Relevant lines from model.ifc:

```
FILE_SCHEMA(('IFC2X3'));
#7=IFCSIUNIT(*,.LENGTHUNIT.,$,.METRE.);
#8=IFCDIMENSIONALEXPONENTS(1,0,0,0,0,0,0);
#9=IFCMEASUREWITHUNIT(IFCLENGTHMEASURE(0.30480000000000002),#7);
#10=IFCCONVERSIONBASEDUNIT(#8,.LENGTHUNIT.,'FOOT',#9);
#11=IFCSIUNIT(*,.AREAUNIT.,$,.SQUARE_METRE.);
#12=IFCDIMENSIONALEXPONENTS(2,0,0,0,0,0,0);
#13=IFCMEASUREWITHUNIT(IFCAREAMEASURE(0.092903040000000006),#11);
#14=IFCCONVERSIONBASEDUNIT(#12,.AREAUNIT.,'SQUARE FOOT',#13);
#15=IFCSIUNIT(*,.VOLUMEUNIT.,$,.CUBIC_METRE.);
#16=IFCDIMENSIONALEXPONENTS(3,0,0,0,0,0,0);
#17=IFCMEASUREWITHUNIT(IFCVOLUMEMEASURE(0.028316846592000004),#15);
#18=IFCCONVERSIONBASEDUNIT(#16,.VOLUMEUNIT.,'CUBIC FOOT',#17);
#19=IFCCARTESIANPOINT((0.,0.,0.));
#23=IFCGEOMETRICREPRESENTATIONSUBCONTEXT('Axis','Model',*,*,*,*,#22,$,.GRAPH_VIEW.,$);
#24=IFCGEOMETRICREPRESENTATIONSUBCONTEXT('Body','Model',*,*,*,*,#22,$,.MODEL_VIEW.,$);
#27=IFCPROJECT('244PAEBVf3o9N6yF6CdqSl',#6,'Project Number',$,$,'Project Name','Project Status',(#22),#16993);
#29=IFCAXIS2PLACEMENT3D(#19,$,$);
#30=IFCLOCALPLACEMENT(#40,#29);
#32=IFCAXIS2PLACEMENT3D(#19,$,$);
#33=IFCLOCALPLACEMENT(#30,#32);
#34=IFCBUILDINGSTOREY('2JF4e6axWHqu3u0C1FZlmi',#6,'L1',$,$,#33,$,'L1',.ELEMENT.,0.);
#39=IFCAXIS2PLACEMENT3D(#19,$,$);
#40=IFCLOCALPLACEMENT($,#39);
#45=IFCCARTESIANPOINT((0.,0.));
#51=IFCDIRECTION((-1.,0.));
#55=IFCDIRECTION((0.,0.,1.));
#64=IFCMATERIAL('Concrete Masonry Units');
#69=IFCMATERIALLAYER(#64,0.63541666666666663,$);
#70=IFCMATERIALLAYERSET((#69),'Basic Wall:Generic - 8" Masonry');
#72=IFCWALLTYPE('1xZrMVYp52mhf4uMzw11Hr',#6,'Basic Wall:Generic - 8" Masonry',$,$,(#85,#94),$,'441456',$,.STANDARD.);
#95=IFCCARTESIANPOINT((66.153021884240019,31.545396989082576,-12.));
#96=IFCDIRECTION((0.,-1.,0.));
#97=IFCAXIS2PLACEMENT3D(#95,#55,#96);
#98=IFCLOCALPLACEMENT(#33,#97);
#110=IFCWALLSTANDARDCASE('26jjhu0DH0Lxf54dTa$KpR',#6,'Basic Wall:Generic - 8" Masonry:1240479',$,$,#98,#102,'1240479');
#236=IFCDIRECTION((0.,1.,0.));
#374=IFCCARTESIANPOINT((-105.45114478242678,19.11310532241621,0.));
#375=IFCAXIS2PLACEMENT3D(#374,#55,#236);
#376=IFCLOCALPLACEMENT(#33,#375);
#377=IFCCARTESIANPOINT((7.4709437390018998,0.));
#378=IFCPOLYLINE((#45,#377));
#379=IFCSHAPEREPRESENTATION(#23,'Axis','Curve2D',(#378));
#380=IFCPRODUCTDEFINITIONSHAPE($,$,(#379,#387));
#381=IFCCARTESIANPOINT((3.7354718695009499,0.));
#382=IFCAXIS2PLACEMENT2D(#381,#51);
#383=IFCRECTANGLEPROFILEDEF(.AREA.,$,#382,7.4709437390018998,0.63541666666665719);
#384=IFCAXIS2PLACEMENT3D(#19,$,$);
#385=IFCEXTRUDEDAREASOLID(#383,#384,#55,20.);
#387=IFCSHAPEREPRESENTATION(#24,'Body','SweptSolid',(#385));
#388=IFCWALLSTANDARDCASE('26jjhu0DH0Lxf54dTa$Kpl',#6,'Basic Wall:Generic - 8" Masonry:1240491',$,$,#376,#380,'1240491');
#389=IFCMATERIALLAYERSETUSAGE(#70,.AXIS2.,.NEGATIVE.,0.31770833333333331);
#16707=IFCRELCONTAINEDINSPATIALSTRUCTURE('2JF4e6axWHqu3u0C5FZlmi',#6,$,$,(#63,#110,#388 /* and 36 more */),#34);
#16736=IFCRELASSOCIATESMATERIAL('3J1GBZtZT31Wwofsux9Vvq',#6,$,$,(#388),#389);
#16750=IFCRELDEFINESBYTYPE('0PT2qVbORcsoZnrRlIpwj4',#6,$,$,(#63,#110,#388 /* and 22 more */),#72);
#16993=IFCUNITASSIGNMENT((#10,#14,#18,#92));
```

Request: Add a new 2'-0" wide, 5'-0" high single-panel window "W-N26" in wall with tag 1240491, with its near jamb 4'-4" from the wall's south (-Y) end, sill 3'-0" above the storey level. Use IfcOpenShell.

```python
import numpy as np
import ifcopenshell
import ifcopenshell.api.feature
import ifcopenshell.api.geometry
import ifcopenshell.api.root
import ifcopenshell.api.spatial
import ifcopenshell.api.type
import ifcopenshell.geom
import ifcopenshell.util.element
import ifcopenshell.util.placement
import ifcopenshell.util.representation
import ifcopenshell.util.shape
import ifcopenshell.util.unit

model = ifcopenshell.open("model.ifc")
unit_scale = ifcopenshell.util.unit.calculate_unit_scale(model)
settings = ifcopenshell.geom.settings()


def volume(element):
    """Net volume in cubic metres, openings subtracted."""
    shape = ifcopenshell.geom.create_shape(settings, element)
    return ifcopenshell.util.shape.get_volume(shape.geometry)


wall = model.by_guid("26jjhu0DH0Lxf54dTa$Kpl")
storey = ifcopenshell.util.element.get_container(wall, ifc_class="IfcBuildingStorey")
context = ifcopenshell.util.representation.get_context(model, "Model", "Body", "MODEL_VIEW")
before = volume(wall)

width, height, from_end, sill = 0.6096, 1.524, 1.3208, 0.9144  # metres

# The wall runs along its own X axis, and the end named is its -X end.
wall_shape = ifcopenshell.geom.create_shape(settings, wall)
x, y, z = ifcopenshell.util.shape.get_vertices(wall_shape.geometry).T
start = x.min() + from_end
face, thickness = float(y.min()), float(y.max() - y.min())
wall_matrix = ifcopenshell.util.placement.get_local_placement(wall.ObjectPlacement)
level = ifcopenshell.util.placement.get_local_placement(storey.ObjectPlacement)[2, 3]


def in_wall(x, y):
    """Placement at x, y metres in the wall's axes, at sill height."""
    matrix = wall_matrix.copy()
    matrix[:, 3] = wall_matrix @ np.array([x / unit_scale, y / unit_scale, 0.0, 1.0])
    matrix[2, 3] = level + sill / unit_scale
    return matrix


# Opening: a box that overshoots both wall faces by 50 mm.
opening = ifcopenshell.api.root.create_entity(model, ifc_class="IfcOpeningElement")
box = ifcopenshell.api.geometry.add_wall_representation(
    model, context=context, length=width, height=height, thickness=thickness + 0.1
)
ifcopenshell.api.geometry.assign_representation(model, product=opening, representation=box)
ifcopenshell.api.geometry.edit_object_placement(model, product=opening, matrix=in_wall(start, face - 0.05), is_si=False)
ifcopenshell.api.feature.add_feature(model, feature=opening, element=wall)

window = ifcopenshell.api.root.create_entity(model, ifc_class="IfcWindow", name="W-N26")
window.OverallWidth, window.OverallHeight = width / unit_scale, height / unit_scale
body = ifcopenshell.api.geometry.add_window_representation(
    model,
    context=context,
    overall_width=window.OverallWidth,
    overall_height=window.OverallHeight,
    partition_type="SINGLE_PANEL",
)
ifcopenshell.api.geometry.assign_representation(model, product=window, representation=body)
ifcopenshell.api.spatial.assign_container(model, products=[window], relating_structure=storey)
fills = ifcopenshell.api.feature.add_filling(model, opening=opening, element=window)
fills.OwnerHistory = window.OwnerHistory  # required in IFC2X3

# IFC2X3 keeps the operation on the window style.
style = ifcopenshell.api.root.create_entity(model, ifc_class="IfcWindowStyle", name="W-N26")
style.OperationType, style.ConstructionType = "SINGLE_PANEL", "NOTDEFINED"
style.ParameterTakesPrecedence = style.Sizeable = False
ifcopenshell.api.type.assign_type(model, related_objects=[window], relating_type=style)

# Centre the window in the wall's thickness.
ifcopenshell.api.geometry.edit_object_placement(model, product=window, matrix=in_wall(start, face), is_si=False)
window_shape = ifcopenshell.geom.create_shape(settings, window)
depth = ifcopenshell.util.shape.get_vertices(window_shape.geometry)[:, 1]
offset = face + thickness / 2 - (depth.min() + depth.max()) / 2
ifcopenshell.api.geometry.edit_object_placement(model, product=window, matrix=in_wall(start, offset), is_si=False)

after = volume(wall)

print(f"wall volume {before:.3f} -> {after:.3f} m3")

model.write("model_updated.ifc")
```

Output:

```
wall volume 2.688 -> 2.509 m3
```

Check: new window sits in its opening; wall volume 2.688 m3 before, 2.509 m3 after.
